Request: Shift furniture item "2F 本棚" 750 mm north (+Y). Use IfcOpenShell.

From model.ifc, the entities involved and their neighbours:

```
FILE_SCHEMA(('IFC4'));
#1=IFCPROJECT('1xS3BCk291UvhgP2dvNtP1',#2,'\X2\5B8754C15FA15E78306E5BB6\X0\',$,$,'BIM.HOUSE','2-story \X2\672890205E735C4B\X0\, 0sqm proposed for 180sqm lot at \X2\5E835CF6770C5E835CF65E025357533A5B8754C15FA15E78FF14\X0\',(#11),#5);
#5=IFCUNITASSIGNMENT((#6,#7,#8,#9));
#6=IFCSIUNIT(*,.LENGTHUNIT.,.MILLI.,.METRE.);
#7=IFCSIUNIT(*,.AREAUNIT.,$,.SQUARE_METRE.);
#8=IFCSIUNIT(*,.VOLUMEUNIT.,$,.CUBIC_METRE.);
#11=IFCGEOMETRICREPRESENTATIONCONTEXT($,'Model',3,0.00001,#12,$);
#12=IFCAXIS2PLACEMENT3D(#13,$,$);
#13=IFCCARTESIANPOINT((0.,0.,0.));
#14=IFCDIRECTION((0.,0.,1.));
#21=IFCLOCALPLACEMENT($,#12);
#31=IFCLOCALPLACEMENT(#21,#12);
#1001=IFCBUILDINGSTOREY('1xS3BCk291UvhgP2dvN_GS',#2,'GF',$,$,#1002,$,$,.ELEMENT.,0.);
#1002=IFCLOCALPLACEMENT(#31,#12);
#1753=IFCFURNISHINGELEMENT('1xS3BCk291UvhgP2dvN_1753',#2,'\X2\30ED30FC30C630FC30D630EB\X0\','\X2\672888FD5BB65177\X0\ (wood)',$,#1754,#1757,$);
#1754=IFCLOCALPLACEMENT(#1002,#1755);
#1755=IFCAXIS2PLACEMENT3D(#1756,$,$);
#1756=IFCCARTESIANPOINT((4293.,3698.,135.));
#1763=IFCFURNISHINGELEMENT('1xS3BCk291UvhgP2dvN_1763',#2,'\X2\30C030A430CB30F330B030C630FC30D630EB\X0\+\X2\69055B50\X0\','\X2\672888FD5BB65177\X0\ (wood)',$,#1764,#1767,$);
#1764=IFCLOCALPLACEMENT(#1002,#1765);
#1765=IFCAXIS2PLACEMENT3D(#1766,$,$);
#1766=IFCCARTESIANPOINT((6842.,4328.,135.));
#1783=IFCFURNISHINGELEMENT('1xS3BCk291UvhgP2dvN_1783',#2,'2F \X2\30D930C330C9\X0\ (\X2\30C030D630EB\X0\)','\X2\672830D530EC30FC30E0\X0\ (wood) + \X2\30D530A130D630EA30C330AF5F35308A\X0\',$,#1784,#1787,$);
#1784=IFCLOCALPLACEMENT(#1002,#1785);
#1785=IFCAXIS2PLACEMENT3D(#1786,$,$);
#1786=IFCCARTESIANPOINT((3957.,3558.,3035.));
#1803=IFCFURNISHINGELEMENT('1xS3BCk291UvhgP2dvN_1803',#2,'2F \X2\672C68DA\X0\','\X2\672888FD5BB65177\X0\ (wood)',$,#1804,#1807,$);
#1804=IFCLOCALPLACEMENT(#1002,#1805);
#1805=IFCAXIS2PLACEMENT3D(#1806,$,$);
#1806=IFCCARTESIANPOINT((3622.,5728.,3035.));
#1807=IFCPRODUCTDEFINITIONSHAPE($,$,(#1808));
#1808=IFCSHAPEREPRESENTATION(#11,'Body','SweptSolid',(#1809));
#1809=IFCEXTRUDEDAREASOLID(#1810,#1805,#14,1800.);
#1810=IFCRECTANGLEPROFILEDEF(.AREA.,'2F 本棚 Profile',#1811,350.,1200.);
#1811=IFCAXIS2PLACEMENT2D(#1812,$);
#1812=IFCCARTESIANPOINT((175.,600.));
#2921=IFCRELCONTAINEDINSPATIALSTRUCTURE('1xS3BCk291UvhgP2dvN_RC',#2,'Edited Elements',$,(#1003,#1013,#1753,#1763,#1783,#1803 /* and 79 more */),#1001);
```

```python
import ifcopenshell
import ifcopenshell.api.geometry
import ifcopenshell.util.placement

model = ifcopenshell.open("model.ifc")

item = model.by_id(1803)
matrix = ifcopenshell.util.placement.get_local_placement(item.ObjectPlacement)
matrix[1, 3] += 750.0
ifcopenshell.api.geometry.edit_object_placement(model, product=item, matrix=matrix, is_si=False)

print(ifcopenshell.util.placement.get_local_placement(item.ObjectPlacement).round(3) + 0.0)

model.write("model_updated.ifc")
```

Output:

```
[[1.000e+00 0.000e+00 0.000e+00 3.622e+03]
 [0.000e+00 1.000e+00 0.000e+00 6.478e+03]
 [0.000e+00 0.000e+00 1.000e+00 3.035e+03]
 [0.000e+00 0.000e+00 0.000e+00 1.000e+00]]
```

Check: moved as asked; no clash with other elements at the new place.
